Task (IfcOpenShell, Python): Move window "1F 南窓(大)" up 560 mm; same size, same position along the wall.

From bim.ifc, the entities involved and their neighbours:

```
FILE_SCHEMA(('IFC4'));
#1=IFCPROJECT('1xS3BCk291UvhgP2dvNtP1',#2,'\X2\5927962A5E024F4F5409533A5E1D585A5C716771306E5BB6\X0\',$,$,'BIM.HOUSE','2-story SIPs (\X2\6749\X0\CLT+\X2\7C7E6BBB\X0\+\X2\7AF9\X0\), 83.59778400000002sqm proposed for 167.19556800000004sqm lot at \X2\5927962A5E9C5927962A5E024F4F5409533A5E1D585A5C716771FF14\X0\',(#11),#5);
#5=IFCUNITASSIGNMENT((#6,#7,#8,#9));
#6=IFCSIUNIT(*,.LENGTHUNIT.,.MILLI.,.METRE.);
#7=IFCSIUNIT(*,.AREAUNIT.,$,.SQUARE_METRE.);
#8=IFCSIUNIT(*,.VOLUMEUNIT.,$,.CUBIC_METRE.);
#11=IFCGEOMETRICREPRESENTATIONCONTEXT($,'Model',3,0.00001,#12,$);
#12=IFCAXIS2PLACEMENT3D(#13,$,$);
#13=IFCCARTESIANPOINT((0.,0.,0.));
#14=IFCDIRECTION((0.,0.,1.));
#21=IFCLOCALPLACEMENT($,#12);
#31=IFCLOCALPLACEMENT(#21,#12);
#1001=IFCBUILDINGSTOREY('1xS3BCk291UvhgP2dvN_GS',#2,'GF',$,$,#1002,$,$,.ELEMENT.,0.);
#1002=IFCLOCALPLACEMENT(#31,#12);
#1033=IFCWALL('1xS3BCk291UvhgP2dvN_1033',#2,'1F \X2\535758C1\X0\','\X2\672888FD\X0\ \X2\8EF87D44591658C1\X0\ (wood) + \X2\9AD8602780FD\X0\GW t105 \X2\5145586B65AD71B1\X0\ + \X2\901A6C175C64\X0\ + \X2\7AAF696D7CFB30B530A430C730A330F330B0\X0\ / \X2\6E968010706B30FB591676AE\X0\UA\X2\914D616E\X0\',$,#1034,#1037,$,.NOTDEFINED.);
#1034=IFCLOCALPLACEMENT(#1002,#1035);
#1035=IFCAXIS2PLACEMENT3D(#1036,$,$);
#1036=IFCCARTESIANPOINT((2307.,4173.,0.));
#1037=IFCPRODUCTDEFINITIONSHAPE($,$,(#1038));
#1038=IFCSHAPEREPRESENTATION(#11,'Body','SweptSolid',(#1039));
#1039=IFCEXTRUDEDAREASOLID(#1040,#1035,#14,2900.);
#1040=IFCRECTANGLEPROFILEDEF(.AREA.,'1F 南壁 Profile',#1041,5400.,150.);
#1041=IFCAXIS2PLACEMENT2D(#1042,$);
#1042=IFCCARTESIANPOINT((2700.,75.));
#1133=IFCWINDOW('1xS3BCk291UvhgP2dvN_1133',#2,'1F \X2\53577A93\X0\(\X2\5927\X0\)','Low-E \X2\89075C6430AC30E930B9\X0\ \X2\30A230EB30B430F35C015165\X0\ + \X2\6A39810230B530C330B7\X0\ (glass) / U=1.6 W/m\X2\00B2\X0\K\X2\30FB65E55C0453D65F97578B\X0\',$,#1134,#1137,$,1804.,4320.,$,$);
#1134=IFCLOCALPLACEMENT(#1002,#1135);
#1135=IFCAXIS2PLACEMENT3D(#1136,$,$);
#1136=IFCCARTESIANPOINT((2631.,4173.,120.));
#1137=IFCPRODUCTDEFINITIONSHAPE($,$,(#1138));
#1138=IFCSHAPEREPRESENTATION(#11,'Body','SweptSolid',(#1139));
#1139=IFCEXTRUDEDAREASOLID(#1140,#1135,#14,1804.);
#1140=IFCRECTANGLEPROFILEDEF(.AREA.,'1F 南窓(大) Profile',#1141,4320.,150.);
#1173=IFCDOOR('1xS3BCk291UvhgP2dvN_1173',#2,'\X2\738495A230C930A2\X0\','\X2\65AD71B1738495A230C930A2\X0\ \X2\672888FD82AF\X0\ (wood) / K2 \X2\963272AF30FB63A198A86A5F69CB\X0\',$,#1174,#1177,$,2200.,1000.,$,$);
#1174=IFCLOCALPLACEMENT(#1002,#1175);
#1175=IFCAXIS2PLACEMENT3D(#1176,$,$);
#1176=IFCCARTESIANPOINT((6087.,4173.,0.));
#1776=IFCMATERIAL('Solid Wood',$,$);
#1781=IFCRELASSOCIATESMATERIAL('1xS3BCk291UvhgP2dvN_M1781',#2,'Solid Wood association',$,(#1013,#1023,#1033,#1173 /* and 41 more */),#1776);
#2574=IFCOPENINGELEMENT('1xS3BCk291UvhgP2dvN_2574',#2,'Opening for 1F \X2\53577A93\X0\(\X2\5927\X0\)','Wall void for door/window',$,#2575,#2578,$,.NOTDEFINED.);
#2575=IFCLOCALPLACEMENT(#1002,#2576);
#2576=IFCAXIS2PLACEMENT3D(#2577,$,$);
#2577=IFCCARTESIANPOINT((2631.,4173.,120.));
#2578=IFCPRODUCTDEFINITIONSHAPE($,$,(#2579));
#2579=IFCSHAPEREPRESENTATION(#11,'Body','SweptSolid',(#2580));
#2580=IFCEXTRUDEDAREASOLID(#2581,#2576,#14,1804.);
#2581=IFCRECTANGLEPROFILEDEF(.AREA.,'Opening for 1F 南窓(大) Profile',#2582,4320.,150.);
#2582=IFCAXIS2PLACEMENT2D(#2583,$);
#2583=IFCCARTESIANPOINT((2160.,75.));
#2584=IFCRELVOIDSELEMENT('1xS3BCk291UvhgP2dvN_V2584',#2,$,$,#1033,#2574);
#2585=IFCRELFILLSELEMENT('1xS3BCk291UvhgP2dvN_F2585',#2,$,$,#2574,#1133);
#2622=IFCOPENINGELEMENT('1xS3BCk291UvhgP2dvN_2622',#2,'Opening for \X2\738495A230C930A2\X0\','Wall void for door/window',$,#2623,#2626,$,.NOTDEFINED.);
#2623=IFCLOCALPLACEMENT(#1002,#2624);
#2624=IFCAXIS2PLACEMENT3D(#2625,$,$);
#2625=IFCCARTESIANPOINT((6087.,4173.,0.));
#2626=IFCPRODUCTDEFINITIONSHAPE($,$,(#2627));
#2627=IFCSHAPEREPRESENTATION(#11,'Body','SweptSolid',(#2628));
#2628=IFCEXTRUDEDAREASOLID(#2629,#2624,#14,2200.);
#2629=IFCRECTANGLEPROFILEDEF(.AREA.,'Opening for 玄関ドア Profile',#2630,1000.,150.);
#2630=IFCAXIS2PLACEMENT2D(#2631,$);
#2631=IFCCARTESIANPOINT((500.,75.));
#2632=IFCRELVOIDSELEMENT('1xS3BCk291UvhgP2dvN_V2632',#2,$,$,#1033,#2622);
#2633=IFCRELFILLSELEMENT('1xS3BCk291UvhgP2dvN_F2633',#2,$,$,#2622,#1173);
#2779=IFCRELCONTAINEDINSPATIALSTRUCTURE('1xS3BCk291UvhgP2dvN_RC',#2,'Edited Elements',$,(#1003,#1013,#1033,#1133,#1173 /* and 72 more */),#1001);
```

```python
import numpy as np
import ifcopenshell
import ifcopenshell.api.geometry
import ifcopenshell.util.placement
import ifcopenshell.util.unit

model = ifcopenshell.open("bim.ifc")
unit_scale = ifcopenshell.util.unit.calculate_unit_scale(model)

window = model.by_guid("1xS3BCk291UvhgP2dvN_1133")
opening = window.FillsVoids[0].RelatingOpeningElement
dz = 560.0

shift = np.array([0.0, 0.0, dz])
# The window is not placed relative to its opening, so move both.
for product in (opening, window):
    matrix = ifcopenshell.util.placement.get_local_placement(product.ObjectPlacement)
    matrix[:3, 3] += shift
    ifcopenshell.api.geometry.edit_object_placement(model, product=product, matrix=matrix, is_si=False)

print(f"moved by {dz * unit_scale:+.3f} m")

model.write("bim_v2.ifc")
```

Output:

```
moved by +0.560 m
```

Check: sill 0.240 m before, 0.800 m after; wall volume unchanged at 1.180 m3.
